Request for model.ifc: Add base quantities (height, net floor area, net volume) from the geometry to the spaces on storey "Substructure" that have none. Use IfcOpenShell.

First a look at what the model holds.

```python
import ifcopenshell
import ifcopenshell.util.element
import ifcopenshell.util.unit

model = ifcopenshell.open("model.ifc")
print(model.schema)
for unit_type in ("LENGTHUNIT", "AREAUNIT", "VOLUMEUNIT"):
    print(unit_type, ifcopenshell.util.unit.calculate_unit_scale(model, unit_type))
storey = next(s for s in model.by_type("IfcBuildingStorey") if s.Name == "Substructure")
spaces = [e for e in ifcopenshell.util.element.get_decomposition(storey) if e.is_a("IfcSpace")]
for e in sorted(spaces, key=lambda e: e.id()):
    print(e.id(), e.is_a(), e.Name, list(ifcopenshell.util.element.get_psets(e, qtos_only=True)), sep=" | ")
```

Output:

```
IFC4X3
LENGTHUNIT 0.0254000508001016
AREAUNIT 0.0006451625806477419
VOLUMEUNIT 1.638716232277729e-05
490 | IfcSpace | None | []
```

```python
import ifcopenshell
import ifcopenshell.api.pset
import ifcopenshell.geom
import ifcopenshell.util.element
import ifcopenshell.util.shape
import ifcopenshell.util.unit

model = ifcopenshell.open("model.ifc")
unit_scale = ifcopenshell.util.unit.calculate_unit_scale(model)
area_scale = ifcopenshell.util.unit.calculate_unit_scale(model, "AREAUNIT")
volume_scale = ifcopenshell.util.unit.calculate_unit_scale(model, "VOLUMEUNIT")
settings = ifcopenshell.geom.settings()

storey = next(s for s in model.by_type("IfcBuildingStorey") if s.Name == "Substructure")
spaces = [e for e in ifcopenshell.util.element.get_decomposition(storey) if e.is_a("IfcSpace")]

for e in sorted(spaces, key=lambda e: e.id()):
    if ifcopenshell.util.element.get_psets(e, qtos_only=True, should_inherit=False):
        continue
    # Geometry comes back in metres, in the element's own axes.
    shape = ifcopenshell.geom.create_shape(settings, e)
    values = {
        "Height": ifcopenshell.util.shape.get_z(shape.geometry) / unit_scale,
        "NetFloorArea": ifcopenshell.util.shape.get_footprint_area(shape.geometry) / area_scale,
        "NetVolume": ifcopenshell.util.shape.get_volume(shape.geometry) / volume_scale,
    }
    qto = ifcopenshell.api.pset.add_qto(model, product=e, name="Qto_SpaceBaseQuantities")
    ifcopenshell.api.pset.edit_qto(model, qto=qto, properties=values)
    print(e.id(), {k: round(v, 3) for k, v in values.items()})

model.write("model-out.ifc")
```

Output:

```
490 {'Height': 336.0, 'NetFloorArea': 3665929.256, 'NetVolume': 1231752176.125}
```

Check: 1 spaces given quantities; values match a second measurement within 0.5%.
